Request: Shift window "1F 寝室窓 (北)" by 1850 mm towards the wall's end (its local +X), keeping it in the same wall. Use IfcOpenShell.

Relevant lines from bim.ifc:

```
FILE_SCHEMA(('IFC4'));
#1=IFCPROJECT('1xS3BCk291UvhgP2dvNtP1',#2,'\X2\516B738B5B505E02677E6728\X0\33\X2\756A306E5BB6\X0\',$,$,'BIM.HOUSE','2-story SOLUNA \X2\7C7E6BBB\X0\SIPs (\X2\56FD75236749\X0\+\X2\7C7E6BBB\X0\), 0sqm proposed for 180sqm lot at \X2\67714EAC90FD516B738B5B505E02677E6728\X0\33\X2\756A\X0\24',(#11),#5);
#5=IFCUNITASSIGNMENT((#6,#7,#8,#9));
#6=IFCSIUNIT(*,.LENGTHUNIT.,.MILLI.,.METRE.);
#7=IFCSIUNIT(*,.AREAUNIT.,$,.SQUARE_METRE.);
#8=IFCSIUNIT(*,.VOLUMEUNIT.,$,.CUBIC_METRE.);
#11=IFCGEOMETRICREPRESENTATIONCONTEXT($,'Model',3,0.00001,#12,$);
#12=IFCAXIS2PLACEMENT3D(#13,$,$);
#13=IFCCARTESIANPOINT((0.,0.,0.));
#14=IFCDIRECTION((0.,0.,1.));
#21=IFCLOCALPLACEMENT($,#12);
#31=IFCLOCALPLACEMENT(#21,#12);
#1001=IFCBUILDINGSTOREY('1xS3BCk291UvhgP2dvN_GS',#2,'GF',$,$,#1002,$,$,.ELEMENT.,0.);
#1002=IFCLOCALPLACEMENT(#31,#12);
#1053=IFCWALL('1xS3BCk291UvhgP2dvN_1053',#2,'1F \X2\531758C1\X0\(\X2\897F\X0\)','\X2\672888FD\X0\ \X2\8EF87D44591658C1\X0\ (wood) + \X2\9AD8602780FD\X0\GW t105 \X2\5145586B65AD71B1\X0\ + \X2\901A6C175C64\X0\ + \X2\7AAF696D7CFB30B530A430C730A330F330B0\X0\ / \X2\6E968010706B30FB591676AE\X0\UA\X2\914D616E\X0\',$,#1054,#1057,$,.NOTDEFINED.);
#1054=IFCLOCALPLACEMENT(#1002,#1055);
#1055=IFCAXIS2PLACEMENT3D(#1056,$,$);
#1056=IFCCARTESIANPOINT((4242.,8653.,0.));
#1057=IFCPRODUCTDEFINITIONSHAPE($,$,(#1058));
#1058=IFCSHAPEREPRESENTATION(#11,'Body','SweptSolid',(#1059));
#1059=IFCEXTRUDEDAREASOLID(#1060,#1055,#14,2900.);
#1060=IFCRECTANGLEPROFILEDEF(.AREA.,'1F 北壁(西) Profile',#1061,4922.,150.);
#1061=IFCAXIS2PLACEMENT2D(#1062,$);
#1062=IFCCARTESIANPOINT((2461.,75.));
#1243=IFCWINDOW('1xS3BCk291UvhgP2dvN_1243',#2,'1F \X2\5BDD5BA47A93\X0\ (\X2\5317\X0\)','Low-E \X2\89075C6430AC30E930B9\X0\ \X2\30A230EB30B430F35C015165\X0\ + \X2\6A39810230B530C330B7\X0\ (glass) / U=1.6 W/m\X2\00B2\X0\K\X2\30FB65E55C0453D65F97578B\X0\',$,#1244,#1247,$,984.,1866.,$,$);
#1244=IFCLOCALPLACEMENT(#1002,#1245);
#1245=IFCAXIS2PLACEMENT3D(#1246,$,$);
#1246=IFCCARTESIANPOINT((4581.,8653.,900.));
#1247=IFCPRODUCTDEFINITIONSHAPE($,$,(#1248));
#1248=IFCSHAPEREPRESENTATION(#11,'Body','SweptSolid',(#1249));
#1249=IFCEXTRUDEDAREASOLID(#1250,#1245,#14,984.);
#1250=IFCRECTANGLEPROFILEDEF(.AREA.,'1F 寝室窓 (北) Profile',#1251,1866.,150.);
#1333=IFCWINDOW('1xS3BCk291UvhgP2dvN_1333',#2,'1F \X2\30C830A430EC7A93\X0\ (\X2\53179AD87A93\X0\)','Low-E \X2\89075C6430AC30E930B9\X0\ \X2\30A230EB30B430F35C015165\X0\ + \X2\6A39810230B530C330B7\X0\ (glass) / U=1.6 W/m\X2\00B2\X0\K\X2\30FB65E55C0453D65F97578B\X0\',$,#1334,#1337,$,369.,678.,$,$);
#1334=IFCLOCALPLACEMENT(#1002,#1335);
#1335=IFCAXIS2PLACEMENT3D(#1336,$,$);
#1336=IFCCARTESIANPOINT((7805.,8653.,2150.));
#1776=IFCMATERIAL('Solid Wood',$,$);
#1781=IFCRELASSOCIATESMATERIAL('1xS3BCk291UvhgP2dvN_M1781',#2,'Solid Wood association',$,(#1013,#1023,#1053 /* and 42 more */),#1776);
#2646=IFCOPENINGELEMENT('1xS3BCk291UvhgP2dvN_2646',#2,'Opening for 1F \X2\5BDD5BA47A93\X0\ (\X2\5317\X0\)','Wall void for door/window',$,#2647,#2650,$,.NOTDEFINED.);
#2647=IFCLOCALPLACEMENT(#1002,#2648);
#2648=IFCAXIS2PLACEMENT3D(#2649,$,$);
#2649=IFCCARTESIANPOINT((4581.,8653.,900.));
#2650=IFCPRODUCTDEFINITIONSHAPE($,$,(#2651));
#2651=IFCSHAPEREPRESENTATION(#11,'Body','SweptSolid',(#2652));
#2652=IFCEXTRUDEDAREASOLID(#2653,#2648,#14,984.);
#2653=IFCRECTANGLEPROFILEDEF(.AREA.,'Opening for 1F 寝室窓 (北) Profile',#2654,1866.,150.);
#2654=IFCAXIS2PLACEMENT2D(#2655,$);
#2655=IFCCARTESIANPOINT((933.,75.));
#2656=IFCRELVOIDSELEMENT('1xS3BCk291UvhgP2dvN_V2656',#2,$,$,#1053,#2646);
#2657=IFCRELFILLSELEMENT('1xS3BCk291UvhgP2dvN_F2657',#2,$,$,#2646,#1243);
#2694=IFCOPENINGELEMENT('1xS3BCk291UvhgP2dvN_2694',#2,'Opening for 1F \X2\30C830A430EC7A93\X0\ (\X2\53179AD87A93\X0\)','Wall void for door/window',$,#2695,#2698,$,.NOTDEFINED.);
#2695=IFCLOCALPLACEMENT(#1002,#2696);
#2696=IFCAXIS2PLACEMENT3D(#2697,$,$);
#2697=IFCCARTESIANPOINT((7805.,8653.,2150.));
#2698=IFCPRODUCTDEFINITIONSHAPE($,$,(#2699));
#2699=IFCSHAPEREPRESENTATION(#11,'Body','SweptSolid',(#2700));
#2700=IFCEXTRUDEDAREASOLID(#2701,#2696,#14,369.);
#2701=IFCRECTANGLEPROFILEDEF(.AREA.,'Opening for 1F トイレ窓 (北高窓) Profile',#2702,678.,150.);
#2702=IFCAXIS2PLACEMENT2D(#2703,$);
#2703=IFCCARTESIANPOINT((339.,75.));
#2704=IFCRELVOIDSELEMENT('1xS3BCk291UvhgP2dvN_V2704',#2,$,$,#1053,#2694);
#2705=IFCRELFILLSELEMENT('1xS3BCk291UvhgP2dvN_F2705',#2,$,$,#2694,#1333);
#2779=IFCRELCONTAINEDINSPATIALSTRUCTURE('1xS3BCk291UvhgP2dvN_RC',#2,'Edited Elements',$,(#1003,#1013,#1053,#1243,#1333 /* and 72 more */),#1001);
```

```python
import ifcopenshell
import ifcopenshell.api.geometry
import ifcopenshell.util.placement
import ifcopenshell.util.unit

model = ifcopenshell.open("bim.ifc")
unit_scale = ifcopenshell.util.unit.calculate_unit_scale(model)

window = model.by_guid("1xS3BCk291UvhgP2dvN_1243")
opening = window.FillsVoids[0].RelatingOpeningElement
wall = opening.VoidsElements[0].RelatingBuildingElement

wall_matrix = ifcopenshell.util.placement.get_local_placement(wall.ObjectPlacement)
shift = wall_matrix[:3, 0] * 1.85 / unit_scale
before = ifcopenshell.util.placement.get_local_placement(window.ObjectPlacement)[:3, 3].copy()

# The window is not placed relative to its opening, so move both.
for product in (opening, window):
    matrix = ifcopenshell.util.placement.get_local_placement(product.ObjectPlacement)
    matrix[:3, 3] += shift
    ifcopenshell.api.geometry.edit_object_placement(model, product=product, matrix=matrix, is_si=False)

after = ifcopenshell.util.placement.get_local_placement(window.ObjectPlacement)[:3, 3]
print("window moved by", (after - before).round(3) + 0.0)

model.write("bim_updated.ifc")
```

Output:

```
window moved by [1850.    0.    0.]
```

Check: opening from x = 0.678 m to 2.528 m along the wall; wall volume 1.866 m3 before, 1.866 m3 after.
